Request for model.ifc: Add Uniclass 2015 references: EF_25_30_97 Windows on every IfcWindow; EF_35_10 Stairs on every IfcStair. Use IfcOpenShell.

First a look at what the model holds.

```python
import ifcopenshell

model = ifcopenshell.open("model.ifc")
print(model.schema)
print("classifications:", [c.Name for c in model.by_type("IfcClassification")])
for ifc_class in ("IfcDoor", "IfcRoof", "IfcStair", "IfcWall", "IfcWindow"):
    print(ifc_class, len(model.by_type(ifc_class)))
```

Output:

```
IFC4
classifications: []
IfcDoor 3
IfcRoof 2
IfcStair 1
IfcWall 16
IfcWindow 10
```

```python
import ifcopenshell
import ifcopenshell.api.classification

model = ifcopenshell.open("model.ifc")

system = ifcopenshell.api.classification.add_classification(model, classification="Uniclass 2015")

codes = {
    "IfcWindow": ("EF_25_30_97", "Windows"),
    "IfcStair": ("EF_35_10", "Stairs"),
}
for ifc_class, (code, name) in codes.items():
    products = model.by_type(ifc_class)
    ifcopenshell.api.classification.add_reference(
        model, products=products, classification=system, identification=code, name=name
    )
    print(code, len(products))

model.write("model_edited.ifc")
```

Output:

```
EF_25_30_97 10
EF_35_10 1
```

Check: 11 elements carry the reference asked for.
